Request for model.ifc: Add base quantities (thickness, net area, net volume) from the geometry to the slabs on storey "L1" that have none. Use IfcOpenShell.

First a look at what the model holds.

```python
import ifcopenshell
import ifcopenshell.util.element
import ifcopenshell.util.unit

model = ifcopenshell.open("model.ifc")
print(model.schema)
for unit_type in ("LENGTHUNIT", "AREAUNIT", "VOLUMEUNIT"):
    print(unit_type, ifcopenshell.util.unit.calculate_unit_scale(model, unit_type))
storey = next(s for s in model.by_type("IfcBuildingStorey") if s.Name == "L1")
slabs = [e for e in ifcopenshell.util.element.get_decomposition(storey) if e.is_a("IfcSlab")]
for e in sorted(slabs, key=lambda e: e.id()):
    print(e.id(), e.is_a(), e.Name, list(ifcopenshell.util.element.get_psets(e, qtos_only=True)), sep=" | ")
```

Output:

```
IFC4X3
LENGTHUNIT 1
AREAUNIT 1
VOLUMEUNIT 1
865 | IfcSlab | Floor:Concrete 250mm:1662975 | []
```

```python
import ifcopenshell
import ifcopenshell.api.pset
import ifcopenshell.geom
import ifcopenshell.util.element
import ifcopenshell.util.shape
import ifcopenshell.util.unit

model = ifcopenshell.open("model.ifc")
unit_scale = ifcopenshell.util.unit.calculate_unit_scale(model)
area_scale = ifcopenshell.util.unit.calculate_unit_scale(model, "AREAUNIT")
volume_scale = ifcopenshell.util.unit.calculate_unit_scale(model, "VOLUMEUNIT")
settings = ifcopenshell.geom.settings()

storey = next(s for s in model.by_type("IfcBuildingStorey") if s.Name == "L1")
slabs = [e for e in ifcopenshell.util.element.get_decomposition(storey) if e.is_a("IfcSlab")]

for e in sorted(slabs, key=lambda e: e.id()):
    if ifcopenshell.util.element.get_psets(e, qtos_only=True, should_inherit=False):
        continue
    # Geometry comes back in metres, in the element's own axes.
    shape = ifcopenshell.geom.create_shape(settings, e)
    values = {
        "Width": ifcopenshell.util.shape.get_z(shape.geometry) / unit_scale,
        "NetArea": ifcopenshell.util.shape.get_footprint_area(shape.geometry) / area_scale,
        "NetVolume": ifcopenshell.util.shape.get_volume(shape.geometry) / volume_scale,
    }
    qto = ifcopenshell.api.pset.add_qto(model, product=e, name="Qto_SlabBaseQuantities")
    ifcopenshell.api.pset.edit_qto(model, qto=qto, properties=values)
    print(e.id(), {k: round(v, 3) for k, v in values.items()})

model.write("model_edited.ifc")
```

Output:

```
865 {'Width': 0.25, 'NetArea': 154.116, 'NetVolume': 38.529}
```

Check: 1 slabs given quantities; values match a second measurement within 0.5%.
